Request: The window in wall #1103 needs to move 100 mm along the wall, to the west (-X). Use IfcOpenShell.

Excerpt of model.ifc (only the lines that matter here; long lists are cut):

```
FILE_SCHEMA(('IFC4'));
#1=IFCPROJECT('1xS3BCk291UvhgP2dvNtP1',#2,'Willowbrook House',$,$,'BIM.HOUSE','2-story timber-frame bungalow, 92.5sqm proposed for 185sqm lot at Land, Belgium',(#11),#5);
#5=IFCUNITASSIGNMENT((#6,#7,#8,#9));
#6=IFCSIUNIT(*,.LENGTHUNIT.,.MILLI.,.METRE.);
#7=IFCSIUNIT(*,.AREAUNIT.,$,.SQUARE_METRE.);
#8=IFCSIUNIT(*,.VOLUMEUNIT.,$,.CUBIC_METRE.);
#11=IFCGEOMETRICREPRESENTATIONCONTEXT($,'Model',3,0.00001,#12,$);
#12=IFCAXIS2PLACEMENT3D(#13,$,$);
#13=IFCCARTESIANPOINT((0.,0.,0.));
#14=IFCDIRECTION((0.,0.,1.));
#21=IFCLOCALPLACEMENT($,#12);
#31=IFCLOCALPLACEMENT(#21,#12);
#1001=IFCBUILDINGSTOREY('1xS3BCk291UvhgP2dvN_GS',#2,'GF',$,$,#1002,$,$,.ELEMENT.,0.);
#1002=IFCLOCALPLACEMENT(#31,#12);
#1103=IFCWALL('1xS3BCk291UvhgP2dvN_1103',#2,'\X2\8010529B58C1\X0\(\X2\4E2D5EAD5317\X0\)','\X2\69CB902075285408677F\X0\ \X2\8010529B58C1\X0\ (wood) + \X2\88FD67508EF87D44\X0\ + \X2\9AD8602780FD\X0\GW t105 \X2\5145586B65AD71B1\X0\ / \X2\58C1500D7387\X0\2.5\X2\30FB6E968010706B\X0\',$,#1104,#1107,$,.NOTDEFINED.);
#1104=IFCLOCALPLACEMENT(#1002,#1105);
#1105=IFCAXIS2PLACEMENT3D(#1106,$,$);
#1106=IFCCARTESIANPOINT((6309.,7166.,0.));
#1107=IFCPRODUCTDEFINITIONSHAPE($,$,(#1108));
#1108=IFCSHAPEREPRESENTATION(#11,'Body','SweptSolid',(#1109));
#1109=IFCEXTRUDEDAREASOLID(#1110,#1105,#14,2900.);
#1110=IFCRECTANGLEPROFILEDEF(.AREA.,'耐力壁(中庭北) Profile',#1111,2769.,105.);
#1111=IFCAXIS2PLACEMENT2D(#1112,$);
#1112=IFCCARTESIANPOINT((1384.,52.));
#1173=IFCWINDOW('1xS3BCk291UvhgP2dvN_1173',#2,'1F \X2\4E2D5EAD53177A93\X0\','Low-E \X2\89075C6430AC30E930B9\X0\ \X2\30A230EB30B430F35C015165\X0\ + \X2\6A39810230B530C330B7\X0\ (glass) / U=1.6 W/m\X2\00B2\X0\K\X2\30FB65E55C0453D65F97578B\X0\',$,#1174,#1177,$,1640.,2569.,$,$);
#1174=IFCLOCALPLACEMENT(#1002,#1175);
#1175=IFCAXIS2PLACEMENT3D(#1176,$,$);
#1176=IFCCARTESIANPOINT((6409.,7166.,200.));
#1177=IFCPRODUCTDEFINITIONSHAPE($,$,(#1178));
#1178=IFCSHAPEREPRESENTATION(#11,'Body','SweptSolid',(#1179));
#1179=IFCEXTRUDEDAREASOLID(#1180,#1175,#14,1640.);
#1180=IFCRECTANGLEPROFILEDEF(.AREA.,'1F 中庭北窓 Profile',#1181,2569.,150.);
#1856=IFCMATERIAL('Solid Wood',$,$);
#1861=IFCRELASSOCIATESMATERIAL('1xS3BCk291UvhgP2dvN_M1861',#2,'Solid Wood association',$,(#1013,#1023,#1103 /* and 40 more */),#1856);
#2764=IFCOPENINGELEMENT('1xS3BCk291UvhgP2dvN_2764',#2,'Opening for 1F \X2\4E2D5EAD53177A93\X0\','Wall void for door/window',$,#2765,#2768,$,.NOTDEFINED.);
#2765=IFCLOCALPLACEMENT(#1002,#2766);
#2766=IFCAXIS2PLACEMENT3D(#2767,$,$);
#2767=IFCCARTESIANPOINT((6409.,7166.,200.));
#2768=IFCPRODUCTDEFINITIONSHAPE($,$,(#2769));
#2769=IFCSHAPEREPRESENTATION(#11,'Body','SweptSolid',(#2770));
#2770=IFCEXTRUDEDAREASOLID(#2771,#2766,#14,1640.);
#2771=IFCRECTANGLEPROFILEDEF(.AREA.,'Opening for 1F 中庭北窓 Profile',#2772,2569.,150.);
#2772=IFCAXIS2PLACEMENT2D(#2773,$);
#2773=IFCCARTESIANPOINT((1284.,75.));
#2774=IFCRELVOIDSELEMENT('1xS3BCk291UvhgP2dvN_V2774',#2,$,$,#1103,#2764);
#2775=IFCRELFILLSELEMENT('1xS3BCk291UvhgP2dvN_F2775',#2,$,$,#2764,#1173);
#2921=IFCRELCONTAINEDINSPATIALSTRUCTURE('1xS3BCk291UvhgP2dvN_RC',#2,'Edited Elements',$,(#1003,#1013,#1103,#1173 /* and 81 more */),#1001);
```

```python
import ifcopenshell
import ifcopenshell.api.geometry
import ifcopenshell.util.placement
import ifcopenshell.util.unit

model = ifcopenshell.open("model.ifc")
unit_scale = ifcopenshell.util.unit.calculate_unit_scale(model)

window = model.by_id(1173)
opening = window.FillsVoids[0].RelatingOpeningElement
wall = opening.VoidsElements[0].RelatingBuildingElement

wall_matrix = ifcopenshell.util.placement.get_local_placement(wall.ObjectPlacement)
shift = wall_matrix[:3, 0] * -0.1 / unit_scale
before = ifcopenshell.util.placement.get_local_placement(window.ObjectPlacement)[:3, 3].copy()

# The window is not placed relative to its opening, so move both.
for product in (opening, window):
    matrix = ifcopenshell.util.placement.get_local_placement(product.ObjectPlacement)
    matrix[:3, 3] += shift
    ifcopenshell.api.geometry.edit_object_placement(model, product=product, matrix=matrix, is_si=False)

after = ifcopenshell.util.placement.get_local_placement(window.ObjectPlacement)[:3, 3]
print("window moved by", (after - before).round(3) + 0.0)

model.write("model_updated.ifc")
```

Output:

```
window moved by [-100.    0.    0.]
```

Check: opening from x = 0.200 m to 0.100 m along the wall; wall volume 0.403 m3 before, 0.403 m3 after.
